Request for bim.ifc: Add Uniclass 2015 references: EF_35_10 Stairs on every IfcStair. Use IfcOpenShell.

First a look at what the model holds.

```python
import ifcopenshell

model = ifcopenshell.open("bim.ifc")
print(model.schema)
print("classifications:", [c.Name for c in model.by_type("IfcClassification")])
for ifc_class in ("IfcDoor", "IfcRoof", "IfcStair", "IfcWall", "IfcWindow"):
    print(ifc_class, len(model.by_type(ifc_class)))
```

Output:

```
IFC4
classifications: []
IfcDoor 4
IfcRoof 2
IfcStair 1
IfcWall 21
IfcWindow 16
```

```python
import ifcopenshell
import ifcopenshell.api.classification

model = ifcopenshell.open("bim.ifc")

system = ifcopenshell.api.classification.add_classification(model, classification="Uniclass 2015")

codes = {
    "IfcStair": ("EF_35_10", "Stairs"),
}
for ifc_class, (code, name) in codes.items():
    products = model.by_type(ifc_class)
    ifcopenshell.api.classification.add_reference(
        model, products=products, classification=system, identification=code, name=name
    )
    print(code, len(products))

model.write("bim_rev.ifc")
```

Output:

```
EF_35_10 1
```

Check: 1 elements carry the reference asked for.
